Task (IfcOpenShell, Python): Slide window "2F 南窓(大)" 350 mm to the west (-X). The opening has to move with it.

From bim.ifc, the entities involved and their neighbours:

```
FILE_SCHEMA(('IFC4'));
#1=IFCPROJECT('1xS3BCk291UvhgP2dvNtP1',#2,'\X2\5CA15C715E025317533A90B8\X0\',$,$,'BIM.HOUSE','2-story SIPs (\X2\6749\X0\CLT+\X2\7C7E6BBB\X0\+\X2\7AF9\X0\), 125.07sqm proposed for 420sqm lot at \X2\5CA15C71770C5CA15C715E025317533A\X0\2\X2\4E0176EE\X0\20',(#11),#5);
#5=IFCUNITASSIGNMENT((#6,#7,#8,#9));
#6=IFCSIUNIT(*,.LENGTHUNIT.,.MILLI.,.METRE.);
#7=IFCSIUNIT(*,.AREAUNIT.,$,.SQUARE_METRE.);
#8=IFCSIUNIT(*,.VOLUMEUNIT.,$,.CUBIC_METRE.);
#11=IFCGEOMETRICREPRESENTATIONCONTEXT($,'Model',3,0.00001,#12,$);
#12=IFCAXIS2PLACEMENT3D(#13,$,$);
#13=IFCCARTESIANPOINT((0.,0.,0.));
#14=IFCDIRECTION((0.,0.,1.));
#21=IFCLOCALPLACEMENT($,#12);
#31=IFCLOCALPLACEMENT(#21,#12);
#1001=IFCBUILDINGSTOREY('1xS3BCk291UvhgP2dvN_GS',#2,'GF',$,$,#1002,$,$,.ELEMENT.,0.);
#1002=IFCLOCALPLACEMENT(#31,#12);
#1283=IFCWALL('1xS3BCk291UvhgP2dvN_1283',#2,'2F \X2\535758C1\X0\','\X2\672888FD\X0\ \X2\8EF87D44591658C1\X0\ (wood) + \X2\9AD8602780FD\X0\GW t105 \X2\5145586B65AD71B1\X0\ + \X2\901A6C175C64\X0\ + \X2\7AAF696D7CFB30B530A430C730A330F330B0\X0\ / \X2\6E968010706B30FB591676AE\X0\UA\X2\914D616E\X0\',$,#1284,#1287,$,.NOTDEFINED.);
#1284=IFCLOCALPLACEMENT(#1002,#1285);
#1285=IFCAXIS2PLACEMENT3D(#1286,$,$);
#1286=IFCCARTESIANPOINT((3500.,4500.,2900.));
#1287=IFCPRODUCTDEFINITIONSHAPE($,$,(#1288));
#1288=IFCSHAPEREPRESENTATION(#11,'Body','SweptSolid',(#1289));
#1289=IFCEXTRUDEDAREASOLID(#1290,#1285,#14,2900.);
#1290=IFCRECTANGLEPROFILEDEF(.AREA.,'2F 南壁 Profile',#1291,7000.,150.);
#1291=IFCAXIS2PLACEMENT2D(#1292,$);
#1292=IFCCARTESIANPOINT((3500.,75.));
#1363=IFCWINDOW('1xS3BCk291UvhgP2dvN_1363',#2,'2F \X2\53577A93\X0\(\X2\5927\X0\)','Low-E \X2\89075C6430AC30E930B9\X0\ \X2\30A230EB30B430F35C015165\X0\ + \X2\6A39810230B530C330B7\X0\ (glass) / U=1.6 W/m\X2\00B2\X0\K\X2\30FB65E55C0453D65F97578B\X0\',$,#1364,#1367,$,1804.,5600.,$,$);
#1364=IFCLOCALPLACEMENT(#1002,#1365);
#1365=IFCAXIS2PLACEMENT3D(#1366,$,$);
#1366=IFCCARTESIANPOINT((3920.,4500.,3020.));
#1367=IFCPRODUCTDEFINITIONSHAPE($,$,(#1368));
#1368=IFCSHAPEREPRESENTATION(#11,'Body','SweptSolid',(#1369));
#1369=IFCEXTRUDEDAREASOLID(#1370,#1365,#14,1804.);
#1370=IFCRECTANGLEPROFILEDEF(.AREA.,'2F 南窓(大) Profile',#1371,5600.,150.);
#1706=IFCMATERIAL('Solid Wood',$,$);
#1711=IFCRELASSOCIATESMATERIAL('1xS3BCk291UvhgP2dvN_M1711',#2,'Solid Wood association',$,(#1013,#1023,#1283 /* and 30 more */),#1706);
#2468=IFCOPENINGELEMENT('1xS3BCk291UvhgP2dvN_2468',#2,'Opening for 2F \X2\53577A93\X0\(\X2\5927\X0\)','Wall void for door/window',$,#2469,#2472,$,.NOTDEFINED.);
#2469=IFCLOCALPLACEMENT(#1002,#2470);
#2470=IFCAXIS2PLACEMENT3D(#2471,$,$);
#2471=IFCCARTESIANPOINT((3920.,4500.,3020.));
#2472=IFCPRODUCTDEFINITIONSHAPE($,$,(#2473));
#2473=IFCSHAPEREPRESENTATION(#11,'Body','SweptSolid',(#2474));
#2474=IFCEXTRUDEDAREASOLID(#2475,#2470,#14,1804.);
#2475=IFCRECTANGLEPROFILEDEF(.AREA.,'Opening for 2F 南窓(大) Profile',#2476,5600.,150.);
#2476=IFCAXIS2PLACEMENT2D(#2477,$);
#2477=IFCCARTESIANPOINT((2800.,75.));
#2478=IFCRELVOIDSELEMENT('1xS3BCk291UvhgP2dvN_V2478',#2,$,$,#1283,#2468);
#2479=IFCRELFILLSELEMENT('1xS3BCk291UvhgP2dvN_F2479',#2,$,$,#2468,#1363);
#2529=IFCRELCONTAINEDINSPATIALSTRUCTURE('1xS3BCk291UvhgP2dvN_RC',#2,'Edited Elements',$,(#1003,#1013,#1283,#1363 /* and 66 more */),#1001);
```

```python
import ifcopenshell
import ifcopenshell.api.geometry
import ifcopenshell.util.placement
import ifcopenshell.util.unit

model = ifcopenshell.open("bim.ifc")
unit_scale = ifcopenshell.util.unit.calculate_unit_scale(model)

window = model.by_guid("1xS3BCk291UvhgP2dvN_1363")
opening = window.FillsVoids[0].RelatingOpeningElement
wall = opening.VoidsElements[0].RelatingBuildingElement

wall_matrix = ifcopenshell.util.placement.get_local_placement(wall.ObjectPlacement)
shift = wall_matrix[:3, 0] * -0.35 / unit_scale
before = ifcopenshell.util.placement.get_local_placement(window.ObjectPlacement)[:3, 3].copy()

# The window is not placed relative to its opening, so move both.
for product in (opening, window):
    matrix = ifcopenshell.util.placement.get_local_placement(product.ObjectPlacement)
    matrix[:3, 3] += shift
    ifcopenshell.api.geometry.edit_object_placement(model, product=product, matrix=matrix, is_si=False)

after = ifcopenshell.util.placement.get_local_placement(window.ObjectPlacement)[:3, 3]
print("window moved by", (after - before).round(3) + 0.0)

model.write("bim_updated.ifc")
```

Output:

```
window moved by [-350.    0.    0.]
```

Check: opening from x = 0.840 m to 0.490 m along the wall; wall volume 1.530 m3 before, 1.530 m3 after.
